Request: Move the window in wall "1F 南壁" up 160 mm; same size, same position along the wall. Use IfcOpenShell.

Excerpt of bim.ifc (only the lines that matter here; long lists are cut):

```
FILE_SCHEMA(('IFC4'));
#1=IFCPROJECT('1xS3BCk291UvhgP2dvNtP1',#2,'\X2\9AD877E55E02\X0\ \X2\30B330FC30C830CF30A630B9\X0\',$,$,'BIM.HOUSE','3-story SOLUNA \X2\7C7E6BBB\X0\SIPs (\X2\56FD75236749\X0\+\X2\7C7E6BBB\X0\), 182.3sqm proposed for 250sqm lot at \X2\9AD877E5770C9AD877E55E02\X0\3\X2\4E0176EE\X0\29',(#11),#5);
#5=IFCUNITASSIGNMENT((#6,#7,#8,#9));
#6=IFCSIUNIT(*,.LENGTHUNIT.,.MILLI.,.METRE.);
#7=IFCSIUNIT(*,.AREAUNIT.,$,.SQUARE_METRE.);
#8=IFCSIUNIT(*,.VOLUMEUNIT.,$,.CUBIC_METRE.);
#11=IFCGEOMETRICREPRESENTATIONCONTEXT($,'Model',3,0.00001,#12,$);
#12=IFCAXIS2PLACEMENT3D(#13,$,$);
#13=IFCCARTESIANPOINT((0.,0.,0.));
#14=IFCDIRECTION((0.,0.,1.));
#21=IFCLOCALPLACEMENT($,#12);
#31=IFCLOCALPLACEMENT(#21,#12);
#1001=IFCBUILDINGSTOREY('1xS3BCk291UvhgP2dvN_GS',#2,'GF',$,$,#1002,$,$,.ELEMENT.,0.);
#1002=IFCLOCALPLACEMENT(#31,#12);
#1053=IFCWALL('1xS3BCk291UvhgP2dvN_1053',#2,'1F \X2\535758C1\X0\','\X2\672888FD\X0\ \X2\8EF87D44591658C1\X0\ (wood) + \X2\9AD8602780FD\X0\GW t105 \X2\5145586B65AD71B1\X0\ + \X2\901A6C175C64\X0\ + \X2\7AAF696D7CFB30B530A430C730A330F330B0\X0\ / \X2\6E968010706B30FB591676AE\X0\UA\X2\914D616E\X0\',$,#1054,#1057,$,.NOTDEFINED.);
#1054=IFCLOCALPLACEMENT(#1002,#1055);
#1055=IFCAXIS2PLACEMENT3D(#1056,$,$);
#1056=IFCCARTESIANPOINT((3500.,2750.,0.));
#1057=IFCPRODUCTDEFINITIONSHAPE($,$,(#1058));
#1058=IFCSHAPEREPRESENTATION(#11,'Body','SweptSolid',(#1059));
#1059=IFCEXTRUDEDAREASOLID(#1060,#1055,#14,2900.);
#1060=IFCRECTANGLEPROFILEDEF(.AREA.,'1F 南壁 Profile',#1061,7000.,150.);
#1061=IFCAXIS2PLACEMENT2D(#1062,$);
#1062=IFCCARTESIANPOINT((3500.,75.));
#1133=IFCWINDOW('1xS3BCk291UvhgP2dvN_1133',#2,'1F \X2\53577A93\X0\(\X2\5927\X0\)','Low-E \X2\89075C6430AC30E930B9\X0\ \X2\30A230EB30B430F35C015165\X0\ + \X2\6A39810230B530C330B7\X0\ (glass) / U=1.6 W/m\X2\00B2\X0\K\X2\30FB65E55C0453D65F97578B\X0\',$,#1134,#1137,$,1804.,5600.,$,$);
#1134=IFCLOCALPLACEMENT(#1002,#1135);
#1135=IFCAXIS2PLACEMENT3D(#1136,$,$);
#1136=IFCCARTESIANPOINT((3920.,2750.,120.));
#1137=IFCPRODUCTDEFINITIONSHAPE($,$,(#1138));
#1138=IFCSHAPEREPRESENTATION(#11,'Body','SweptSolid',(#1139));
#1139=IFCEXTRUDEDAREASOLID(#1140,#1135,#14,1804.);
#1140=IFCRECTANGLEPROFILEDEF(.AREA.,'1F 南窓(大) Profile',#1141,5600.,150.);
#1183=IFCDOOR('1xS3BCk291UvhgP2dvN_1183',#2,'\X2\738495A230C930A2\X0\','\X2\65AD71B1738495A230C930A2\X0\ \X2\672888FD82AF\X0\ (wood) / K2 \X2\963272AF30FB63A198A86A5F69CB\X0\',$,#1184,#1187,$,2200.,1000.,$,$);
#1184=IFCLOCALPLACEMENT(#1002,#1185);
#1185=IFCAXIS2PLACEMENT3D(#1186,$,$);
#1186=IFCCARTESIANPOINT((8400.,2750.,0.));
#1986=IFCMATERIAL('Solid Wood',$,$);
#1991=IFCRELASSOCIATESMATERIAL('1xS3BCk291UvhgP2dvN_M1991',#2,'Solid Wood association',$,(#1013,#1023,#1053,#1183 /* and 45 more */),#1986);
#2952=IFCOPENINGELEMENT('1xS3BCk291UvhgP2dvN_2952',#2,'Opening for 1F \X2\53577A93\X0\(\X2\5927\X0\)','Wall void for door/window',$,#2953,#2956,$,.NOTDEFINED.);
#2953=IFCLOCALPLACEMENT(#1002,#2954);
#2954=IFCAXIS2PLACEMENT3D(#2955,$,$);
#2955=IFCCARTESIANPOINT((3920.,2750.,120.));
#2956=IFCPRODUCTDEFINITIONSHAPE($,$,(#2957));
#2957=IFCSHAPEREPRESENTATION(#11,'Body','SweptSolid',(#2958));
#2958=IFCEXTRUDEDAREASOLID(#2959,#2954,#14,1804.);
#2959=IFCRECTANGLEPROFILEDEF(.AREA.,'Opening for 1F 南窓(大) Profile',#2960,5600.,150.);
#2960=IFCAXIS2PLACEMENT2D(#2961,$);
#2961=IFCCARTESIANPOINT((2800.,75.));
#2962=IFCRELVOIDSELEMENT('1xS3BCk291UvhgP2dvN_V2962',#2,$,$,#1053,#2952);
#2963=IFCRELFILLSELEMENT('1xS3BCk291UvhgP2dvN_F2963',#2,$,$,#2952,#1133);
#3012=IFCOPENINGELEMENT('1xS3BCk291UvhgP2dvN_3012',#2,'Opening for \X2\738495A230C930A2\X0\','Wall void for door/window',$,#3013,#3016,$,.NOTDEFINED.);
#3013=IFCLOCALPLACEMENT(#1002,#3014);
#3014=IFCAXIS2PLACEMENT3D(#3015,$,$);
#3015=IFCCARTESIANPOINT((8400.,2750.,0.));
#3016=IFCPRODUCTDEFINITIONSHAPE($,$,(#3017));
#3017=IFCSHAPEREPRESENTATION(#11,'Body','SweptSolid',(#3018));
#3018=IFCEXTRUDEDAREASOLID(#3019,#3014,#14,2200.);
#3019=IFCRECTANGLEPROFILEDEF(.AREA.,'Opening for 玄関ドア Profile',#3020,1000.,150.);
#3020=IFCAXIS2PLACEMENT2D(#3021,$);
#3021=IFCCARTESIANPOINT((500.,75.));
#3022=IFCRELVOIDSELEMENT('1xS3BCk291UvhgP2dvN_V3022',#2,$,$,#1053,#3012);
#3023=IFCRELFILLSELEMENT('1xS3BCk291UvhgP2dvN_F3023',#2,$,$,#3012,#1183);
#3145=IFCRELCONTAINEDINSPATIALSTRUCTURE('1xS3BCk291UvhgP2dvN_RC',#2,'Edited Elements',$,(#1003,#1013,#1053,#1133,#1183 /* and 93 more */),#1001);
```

```python
import numpy as np
import ifcopenshell
import ifcopenshell.api.geometry
import ifcopenshell.util.placement
import ifcopenshell.util.unit

model = ifcopenshell.open("bim.ifc")
unit_scale = ifcopenshell.util.unit.calculate_unit_scale(model)

window = model.by_guid("1xS3BCk291UvhgP2dvN_1133")
opening = window.FillsVoids[0].RelatingOpeningElement
dz = 160.0

shift = np.array([0.0, 0.0, dz])
# The window is not placed relative to its opening, so move both.
for product in (opening, window):
    matrix = ifcopenshell.util.placement.get_local_placement(product.ObjectPlacement)
    matrix[:3, 3] += shift
    ifcopenshell.api.geometry.edit_object_placement(model, product=product, matrix=matrix, is_si=False)

print(f"moved by {dz * unit_scale:+.3f} m")

model.write("bim_rev.ifc")
```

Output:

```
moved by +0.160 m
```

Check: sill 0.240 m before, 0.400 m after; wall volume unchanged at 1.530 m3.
